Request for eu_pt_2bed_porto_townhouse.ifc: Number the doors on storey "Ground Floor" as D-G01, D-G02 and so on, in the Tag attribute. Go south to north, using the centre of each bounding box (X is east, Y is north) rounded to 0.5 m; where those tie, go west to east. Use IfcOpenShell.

First a look at what the model holds.

```python
import ifcopenshell
import ifcopenshell.util.element
import ifcopenshell.util.placement

model = ifcopenshell.open("eu_pt_2bed_porto_townhouse.ifc")
print(model.schema)
storey = next(s for s in model.by_type("IfcBuildingStorey") if s.Name == "Ground Floor")
doors = [e for e in ifcopenshell.util.element.get_decomposition(storey) if e.is_a("IfcDoor")]
for e in sorted(doors, key=lambda e: e.id()):
    origin = ifcopenshell.util.placement.get_local_placement(e.ObjectPlacement)[:3, 3]
    print(e.id(), e.Tag, e.Name, origin.round(2) + 0.0, sep=" | ")
```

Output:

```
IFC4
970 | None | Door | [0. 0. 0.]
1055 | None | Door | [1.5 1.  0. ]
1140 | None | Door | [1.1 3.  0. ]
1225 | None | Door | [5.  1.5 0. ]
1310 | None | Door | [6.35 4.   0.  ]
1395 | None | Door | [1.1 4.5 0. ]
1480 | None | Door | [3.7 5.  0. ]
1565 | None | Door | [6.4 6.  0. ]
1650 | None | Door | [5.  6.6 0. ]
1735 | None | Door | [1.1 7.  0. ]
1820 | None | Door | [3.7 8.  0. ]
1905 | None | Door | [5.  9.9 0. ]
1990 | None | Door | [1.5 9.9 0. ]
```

```python
import ifcopenshell
import ifcopenshell.geom
import ifcopenshell.util.element
import ifcopenshell.util.shape

model = ifcopenshell.open("eu_pt_2bed_porto_townhouse.ifc")
settings = ifcopenshell.geom.settings()
settings.set("use-world-coords", True)


def centre(element):
    shape = ifcopenshell.geom.create_shape(settings, element)
    return ifcopenshell.util.shape.get_bbox_centroid(shape.geometry)


storey = next(s for s in model.by_type("IfcBuildingStorey") if s.Name == "Ground Floor")
doors = [e for e in ifcopenshell.util.element.get_decomposition(storey) if e.is_a("IfcDoor")]

# Insertion points can sit at a corner or the storey origin, so sort by the geometry (in metres).
centres = {e: centre(e) for e in doors}
doors.sort(key=lambda e: (round(centres[e][1] / 0.5), centres[e][0]))

for i, e in enumerate(doors, start=1):
    number = f"D-G{i:02d}"
    e.Tag = number
    print(e.id(), number)

model.write("eu_pt_2bed_porto_townhouse_v2.ifc")
```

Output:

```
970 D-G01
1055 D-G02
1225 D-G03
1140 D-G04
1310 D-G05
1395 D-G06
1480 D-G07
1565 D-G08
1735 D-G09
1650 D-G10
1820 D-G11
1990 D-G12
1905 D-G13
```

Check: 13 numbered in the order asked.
